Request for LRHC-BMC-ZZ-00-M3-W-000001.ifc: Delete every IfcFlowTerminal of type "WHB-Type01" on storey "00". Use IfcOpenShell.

First a look at what the model holds.

```python
import ifcopenshell
import ifcopenshell.util.element

model = ifcopenshell.open("LRHC-BMC-ZZ-00-M3-W-000001.ifc")
print(model.schema)
storey = next(s for s in model.by_type("IfcBuildingStorey") if s.Name == "00")
terminals = [e for e in ifcopenshell.util.element.get_decomposition(storey) if e.is_a("IfcFlowTerminal")]
seen = {}
for e in terminals:
    element_type = ifcopenshell.util.element.get_type(e)
    name = element_type.Name if element_type not in (None, e) else None
    seen[name] = seen.get(name, 0) + 1
for name, count in sorted(seen.items(), key=str):
    print(count, "x", name)
```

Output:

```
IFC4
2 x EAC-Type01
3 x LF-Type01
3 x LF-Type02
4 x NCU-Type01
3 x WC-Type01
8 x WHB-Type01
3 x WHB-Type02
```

```python
import ifcopenshell
import ifcopenshell.api.root
import ifcopenshell.util.element

model = ifcopenshell.open("LRHC-BMC-ZZ-00-M3-W-000001.ifc")

storey = next(s for s in model.by_type("IfcBuildingStorey") if s.Name == "00")
terminals = [e for e in ifcopenshell.util.element.get_decomposition(storey) if e.is_a("IfcFlowTerminal")]
targets = [e for e in terminals if (t := ifcopenshell.util.element.get_type(e)) not in (None, e) and t.Name == "WHB-Type01"]

for e in targets:
    ifcopenshell.api.root.remove_product(model, product=e)
print(len(targets), "removed")

model.write("LRHC-BMC-ZZ-00-M3-W-000001_v2.ifc")
```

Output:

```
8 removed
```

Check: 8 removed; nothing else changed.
